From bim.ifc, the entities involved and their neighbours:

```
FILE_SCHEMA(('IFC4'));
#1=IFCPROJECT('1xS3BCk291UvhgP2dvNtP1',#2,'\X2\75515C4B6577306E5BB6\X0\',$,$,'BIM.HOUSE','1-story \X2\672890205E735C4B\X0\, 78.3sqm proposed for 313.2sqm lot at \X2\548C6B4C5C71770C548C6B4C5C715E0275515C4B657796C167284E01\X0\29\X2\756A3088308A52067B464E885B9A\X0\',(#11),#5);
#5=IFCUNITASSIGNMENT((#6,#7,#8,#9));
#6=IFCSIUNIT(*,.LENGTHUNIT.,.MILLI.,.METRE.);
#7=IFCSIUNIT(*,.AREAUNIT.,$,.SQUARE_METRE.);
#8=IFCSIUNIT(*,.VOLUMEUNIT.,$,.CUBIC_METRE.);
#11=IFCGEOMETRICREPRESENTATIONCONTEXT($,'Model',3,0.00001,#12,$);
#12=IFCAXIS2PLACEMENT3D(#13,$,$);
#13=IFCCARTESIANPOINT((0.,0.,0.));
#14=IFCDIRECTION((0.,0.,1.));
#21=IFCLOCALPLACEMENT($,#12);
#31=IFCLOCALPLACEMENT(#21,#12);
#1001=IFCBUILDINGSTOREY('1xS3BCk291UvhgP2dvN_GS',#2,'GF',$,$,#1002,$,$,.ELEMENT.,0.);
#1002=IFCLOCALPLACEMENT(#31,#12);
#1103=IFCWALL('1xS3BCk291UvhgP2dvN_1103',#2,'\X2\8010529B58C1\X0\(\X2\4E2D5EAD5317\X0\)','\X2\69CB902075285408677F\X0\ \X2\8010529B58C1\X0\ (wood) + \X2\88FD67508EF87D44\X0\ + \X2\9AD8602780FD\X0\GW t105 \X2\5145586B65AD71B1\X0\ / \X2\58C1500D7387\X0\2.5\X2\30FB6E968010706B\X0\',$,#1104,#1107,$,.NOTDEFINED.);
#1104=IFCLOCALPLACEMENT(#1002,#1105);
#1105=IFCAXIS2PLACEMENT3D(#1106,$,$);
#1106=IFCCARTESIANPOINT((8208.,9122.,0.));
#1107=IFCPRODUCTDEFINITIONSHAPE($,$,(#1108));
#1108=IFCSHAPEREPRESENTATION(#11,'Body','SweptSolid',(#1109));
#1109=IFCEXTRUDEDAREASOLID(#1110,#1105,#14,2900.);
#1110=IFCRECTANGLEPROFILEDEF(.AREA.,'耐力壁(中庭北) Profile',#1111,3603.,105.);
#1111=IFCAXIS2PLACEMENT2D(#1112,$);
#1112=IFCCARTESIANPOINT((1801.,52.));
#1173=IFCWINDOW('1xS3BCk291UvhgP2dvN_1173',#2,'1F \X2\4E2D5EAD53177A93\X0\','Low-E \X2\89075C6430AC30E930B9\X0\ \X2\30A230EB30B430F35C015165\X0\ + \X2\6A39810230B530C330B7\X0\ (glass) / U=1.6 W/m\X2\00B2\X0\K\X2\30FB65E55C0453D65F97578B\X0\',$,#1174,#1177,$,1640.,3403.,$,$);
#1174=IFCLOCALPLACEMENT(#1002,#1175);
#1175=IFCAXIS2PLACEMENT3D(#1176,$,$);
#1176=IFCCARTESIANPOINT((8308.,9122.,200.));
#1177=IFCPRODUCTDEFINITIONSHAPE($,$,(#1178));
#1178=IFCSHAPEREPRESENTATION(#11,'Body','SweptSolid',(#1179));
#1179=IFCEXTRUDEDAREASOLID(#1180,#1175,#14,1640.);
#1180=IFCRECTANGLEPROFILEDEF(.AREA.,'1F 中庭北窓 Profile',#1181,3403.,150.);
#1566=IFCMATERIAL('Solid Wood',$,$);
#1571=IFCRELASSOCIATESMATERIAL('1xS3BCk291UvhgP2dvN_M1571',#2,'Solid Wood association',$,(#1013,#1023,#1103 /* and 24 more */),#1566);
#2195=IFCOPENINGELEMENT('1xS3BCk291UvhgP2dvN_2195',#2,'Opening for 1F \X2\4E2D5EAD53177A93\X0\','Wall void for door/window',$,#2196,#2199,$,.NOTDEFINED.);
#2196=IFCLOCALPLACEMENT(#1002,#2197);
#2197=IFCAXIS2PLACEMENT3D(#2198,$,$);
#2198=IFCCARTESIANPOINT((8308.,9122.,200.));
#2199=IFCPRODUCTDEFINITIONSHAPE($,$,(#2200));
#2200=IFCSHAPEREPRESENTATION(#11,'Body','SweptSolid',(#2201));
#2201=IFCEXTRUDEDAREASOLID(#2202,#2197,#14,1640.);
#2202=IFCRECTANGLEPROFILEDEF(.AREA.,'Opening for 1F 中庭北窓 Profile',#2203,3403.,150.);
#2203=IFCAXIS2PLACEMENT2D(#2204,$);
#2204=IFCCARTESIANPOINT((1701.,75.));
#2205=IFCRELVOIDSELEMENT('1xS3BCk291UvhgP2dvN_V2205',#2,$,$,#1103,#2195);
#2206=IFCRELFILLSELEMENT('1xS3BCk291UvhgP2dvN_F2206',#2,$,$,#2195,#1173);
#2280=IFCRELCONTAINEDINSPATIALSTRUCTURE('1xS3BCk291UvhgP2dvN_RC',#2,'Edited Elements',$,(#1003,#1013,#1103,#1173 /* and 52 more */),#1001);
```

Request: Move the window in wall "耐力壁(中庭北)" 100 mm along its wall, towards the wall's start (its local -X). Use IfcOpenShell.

```python
import ifcopenshell
import ifcopenshell.api.geometry
import ifcopenshell.util.placement
import ifcopenshell.util.unit

model = ifcopenshell.open("bim.ifc")
unit_scale = ifcopenshell.util.unit.calculate_unit_scale(model)

window = model.by_guid("1xS3BCk291UvhgP2dvN_1173")
opening = window.FillsVoids[0].RelatingOpeningElement
wall = opening.VoidsElements[0].RelatingBuildingElement

wall_matrix = ifcopenshell.util.placement.get_local_placement(wall.ObjectPlacement)
shift = wall_matrix[:3, 0] * -0.1 / unit_scale
before = ifcopenshell.util.placement.get_local_placement(window.ObjectPlacement)[:3, 3].copy()

# The window is not placed relative to its opening, so move both.
for product in (opening, window):
    matrix = ifcopenshell.util.placement.get_local_placement(product.ObjectPlacement)
    matrix[:3, 3] += shift
    ifcopenshell.api.geometry.edit_object_placement(model, product=product, matrix=matrix, is_si=False)

after = ifcopenshell.util.placement.get_local_placement(window.ObjectPlacement)[:3, 3]
print("window moved by", (after - before).round(3) + 0.0)

model.write("bim_updated.ifc")
```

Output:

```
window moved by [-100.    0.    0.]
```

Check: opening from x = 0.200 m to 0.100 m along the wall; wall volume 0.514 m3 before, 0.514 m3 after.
